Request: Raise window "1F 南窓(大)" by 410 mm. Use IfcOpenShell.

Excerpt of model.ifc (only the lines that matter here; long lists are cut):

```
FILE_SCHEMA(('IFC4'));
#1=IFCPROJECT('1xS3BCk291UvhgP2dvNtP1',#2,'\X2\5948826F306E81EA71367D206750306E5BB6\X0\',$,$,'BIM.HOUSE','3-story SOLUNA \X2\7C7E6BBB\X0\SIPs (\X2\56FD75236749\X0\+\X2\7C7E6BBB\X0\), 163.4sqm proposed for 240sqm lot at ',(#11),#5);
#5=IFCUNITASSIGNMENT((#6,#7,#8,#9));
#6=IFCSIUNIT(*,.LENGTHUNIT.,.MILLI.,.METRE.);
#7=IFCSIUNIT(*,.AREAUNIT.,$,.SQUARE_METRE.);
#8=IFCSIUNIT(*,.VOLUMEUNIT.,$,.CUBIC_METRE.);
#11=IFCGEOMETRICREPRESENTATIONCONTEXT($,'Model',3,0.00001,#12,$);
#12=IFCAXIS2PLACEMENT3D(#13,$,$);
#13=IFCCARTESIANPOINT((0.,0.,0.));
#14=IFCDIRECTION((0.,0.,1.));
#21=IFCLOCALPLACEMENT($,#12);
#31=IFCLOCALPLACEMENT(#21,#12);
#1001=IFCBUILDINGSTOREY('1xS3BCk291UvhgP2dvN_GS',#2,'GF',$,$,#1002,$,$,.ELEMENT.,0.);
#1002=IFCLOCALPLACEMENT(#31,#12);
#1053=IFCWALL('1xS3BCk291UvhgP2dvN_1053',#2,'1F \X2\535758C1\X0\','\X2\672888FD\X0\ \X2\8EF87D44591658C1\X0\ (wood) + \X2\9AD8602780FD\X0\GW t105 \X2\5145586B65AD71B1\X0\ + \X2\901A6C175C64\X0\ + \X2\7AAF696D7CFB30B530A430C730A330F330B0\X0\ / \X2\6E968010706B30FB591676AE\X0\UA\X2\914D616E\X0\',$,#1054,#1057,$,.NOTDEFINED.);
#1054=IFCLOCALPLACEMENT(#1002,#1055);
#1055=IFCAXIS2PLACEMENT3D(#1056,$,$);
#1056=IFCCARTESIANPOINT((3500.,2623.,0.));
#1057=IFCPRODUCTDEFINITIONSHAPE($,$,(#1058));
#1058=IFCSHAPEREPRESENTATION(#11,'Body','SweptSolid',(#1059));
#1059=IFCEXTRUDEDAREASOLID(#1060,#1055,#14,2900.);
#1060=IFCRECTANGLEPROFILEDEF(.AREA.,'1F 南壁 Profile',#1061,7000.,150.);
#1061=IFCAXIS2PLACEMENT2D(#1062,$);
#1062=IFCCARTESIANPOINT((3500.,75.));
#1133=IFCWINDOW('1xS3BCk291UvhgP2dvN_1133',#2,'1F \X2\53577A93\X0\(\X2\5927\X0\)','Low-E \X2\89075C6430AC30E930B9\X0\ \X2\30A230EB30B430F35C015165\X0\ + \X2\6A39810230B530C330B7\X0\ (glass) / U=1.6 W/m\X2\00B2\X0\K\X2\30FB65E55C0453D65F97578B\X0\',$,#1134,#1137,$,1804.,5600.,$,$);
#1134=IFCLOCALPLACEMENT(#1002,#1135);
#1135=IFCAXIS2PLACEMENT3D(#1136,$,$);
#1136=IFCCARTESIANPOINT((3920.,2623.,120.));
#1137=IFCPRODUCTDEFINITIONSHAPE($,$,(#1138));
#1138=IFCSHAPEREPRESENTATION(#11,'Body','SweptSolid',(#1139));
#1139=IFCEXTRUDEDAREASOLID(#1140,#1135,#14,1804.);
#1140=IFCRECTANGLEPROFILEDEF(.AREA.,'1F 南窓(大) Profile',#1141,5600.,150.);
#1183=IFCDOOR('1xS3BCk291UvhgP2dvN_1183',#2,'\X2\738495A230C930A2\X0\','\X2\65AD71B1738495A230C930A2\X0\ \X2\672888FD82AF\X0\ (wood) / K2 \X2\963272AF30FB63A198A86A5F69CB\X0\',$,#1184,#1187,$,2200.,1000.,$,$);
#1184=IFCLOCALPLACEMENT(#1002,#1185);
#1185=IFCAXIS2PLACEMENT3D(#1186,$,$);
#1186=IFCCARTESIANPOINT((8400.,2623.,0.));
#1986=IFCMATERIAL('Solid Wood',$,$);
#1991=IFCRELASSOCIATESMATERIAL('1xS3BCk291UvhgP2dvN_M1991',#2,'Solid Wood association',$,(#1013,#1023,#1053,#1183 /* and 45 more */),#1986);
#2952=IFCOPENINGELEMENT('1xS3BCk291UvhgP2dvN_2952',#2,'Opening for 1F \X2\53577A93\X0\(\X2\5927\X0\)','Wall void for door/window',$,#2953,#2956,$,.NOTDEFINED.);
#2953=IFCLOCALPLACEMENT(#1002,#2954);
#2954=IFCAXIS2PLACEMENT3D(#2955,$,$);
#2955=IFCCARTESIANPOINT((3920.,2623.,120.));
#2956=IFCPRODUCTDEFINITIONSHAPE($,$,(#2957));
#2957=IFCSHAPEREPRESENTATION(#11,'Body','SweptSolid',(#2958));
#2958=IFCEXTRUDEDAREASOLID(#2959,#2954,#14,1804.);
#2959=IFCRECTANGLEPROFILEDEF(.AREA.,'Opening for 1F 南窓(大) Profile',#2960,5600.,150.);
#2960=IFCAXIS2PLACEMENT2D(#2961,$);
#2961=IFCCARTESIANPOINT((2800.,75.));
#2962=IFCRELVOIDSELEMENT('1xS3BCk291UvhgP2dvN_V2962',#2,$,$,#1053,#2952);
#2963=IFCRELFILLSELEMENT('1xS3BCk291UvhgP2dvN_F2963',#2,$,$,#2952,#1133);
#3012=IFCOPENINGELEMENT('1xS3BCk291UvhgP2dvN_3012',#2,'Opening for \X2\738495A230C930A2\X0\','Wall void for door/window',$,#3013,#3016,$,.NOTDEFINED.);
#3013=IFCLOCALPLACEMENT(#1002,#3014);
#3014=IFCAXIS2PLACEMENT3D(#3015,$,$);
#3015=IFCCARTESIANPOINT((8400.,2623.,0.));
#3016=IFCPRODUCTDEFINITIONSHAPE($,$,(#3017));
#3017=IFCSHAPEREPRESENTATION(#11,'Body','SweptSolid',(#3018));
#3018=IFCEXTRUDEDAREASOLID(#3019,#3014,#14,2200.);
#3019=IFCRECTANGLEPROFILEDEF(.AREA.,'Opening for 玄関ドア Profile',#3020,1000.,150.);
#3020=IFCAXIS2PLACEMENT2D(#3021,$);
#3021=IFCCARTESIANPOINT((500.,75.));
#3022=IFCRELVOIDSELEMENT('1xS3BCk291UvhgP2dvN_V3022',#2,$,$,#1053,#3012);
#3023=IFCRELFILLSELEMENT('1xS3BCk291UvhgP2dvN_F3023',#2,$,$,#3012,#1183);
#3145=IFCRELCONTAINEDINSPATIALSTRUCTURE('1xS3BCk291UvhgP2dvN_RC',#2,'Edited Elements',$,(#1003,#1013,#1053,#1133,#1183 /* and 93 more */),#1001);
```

```python
import numpy as np
import ifcopenshell
import ifcopenshell.api.geometry
import ifcopenshell.util.placement
import ifcopenshell.util.unit

model = ifcopenshell.open("model.ifc")
unit_scale = ifcopenshell.util.unit.calculate_unit_scale(model)

window = model.by_id(1133)
opening = window.FillsVoids[0].RelatingOpeningElement
dz = 410.0

shift = np.array([0.0, 0.0, dz])
# The window is not placed relative to its opening, so move both.
for product in (opening, window):
    matrix = ifcopenshell.util.placement.get_local_placement(product.ObjectPlacement)
    matrix[:3, 3] += shift
    ifcopenshell.api.geometry.edit_object_placement(model, product=product, matrix=matrix, is_si=False)

print(f"moved by {dz * unit_scale:+.3f} m")

model.write("model_v2.ifc")
```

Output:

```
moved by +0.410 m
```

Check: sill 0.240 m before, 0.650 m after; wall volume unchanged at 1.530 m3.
